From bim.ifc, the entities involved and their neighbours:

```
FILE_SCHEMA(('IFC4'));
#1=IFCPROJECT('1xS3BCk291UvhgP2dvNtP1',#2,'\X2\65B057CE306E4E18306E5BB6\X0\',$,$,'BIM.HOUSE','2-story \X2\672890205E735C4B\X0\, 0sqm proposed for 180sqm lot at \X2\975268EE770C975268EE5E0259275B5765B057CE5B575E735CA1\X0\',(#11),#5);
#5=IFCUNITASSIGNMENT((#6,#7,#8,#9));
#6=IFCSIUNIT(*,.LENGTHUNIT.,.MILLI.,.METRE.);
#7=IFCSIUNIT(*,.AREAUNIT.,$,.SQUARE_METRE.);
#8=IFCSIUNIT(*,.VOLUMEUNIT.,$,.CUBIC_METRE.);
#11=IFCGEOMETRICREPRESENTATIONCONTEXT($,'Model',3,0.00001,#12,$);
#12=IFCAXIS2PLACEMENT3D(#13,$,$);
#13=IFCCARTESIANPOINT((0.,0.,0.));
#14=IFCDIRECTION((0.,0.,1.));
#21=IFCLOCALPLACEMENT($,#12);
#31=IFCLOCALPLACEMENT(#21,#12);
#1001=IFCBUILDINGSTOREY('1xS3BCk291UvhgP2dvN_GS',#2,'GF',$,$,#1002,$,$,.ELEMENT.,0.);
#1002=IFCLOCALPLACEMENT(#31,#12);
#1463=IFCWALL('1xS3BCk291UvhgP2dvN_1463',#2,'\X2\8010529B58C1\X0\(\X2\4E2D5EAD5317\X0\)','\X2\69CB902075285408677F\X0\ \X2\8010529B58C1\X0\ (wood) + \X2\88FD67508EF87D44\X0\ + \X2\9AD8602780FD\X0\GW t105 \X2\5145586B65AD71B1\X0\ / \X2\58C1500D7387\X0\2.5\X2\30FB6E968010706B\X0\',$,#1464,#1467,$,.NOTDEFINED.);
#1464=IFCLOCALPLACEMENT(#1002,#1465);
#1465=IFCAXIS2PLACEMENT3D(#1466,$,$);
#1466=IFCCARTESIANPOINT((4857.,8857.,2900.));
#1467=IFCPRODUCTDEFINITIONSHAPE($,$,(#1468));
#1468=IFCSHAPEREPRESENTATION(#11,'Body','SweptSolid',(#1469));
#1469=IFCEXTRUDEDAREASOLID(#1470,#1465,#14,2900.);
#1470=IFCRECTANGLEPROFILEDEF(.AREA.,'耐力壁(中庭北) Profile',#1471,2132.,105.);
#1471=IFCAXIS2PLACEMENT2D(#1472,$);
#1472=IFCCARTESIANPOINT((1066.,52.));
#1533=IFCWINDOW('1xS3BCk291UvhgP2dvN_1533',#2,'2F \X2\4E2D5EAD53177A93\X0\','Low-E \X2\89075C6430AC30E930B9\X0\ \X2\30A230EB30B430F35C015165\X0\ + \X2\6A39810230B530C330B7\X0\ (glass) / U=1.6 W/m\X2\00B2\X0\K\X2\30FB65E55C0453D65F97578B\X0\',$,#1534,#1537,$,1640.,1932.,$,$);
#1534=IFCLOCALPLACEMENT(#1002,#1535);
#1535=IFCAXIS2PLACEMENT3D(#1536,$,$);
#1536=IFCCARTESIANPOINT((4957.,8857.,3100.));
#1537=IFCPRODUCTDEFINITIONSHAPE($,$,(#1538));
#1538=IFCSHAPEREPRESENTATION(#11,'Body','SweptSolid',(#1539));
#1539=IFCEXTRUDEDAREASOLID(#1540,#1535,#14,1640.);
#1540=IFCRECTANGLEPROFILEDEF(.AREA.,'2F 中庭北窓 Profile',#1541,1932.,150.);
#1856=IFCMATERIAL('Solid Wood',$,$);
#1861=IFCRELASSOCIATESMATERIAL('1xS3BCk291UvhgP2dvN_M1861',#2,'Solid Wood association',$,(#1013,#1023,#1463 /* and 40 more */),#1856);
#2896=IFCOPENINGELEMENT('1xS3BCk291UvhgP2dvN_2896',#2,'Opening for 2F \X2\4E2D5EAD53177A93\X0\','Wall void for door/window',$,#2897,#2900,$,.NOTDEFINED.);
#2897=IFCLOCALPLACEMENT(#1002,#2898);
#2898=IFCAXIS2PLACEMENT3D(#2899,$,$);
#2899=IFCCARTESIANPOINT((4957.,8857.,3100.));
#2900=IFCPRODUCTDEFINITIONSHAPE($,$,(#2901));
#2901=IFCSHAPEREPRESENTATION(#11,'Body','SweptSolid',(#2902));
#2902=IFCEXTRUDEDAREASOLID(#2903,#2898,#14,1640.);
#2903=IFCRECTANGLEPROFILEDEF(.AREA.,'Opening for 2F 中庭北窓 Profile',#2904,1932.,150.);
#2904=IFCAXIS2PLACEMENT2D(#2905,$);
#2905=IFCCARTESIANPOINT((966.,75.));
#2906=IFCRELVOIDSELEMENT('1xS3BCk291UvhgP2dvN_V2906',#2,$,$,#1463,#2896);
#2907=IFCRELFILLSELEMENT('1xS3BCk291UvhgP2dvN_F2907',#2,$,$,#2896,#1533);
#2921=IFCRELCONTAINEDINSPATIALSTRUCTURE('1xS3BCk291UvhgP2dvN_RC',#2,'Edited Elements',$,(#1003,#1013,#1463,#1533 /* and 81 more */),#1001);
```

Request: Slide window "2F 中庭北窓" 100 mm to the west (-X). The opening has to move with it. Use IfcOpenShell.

```python
import ifcopenshell
import ifcopenshell.api.geometry
import ifcopenshell.util.placement

model = ifcopenshell.open("bim.ifc")

window = model.by_id(1533)
opening = window.FillsVoids[0].RelatingOpeningElement
wall = opening.VoidsElements[0].RelatingBuildingElement

wall_matrix = ifcopenshell.util.placement.get_local_placement(wall.ObjectPlacement)
shift = wall_matrix[:3, 0] * -100.0
before = ifcopenshell.util.placement.get_local_placement(window.ObjectPlacement)[:3, 3].copy()

# The window is not placed relative to its opening, so move both.
for product in (opening, window):
    matrix = ifcopenshell.util.placement.get_local_placement(product.ObjectPlacement)
    matrix[:3, 3] += shift
    ifcopenshell.api.geometry.edit_object_placement(model, product=product, matrix=matrix, is_si=False)

after = ifcopenshell.util.placement.get_local_placement(window.ObjectPlacement)[:3, 3]
print("window moved by", (after - before).round(3) + 0.0)

model.write("bim_updated.ifc")
```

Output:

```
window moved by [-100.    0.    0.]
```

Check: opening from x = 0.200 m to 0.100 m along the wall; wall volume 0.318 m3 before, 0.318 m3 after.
